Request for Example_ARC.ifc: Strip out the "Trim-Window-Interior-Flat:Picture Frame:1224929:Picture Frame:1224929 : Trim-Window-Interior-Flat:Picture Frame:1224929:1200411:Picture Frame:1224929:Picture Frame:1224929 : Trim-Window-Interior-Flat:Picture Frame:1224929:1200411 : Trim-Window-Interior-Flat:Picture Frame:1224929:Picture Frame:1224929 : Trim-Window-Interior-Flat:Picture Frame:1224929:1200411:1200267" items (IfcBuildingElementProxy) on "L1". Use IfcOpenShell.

First a look at what the model holds.

```python
import ifcopenshell
import ifcopenshell.util.element

model = ifcopenshell.open("Example_ARC.ifc")
print(model.schema)
storey = next(s for s in model.by_type("IfcBuildingStorey") if s.Name == "L1")
proxies = [e for e in ifcopenshell.util.element.get_decomposition(storey) if e.is_a("IfcBuildingElementProxy")]
seen = {}
for e in proxies:
    element_type = ifcopenshell.util.element.get_type(e)
    name = element_type.Name if element_type not in (None, e) else None
    seen[name] = seen.get(name, 0) + 1
for name, count in sorted(seen.items(), key=str):
    print(count, "x", name)
```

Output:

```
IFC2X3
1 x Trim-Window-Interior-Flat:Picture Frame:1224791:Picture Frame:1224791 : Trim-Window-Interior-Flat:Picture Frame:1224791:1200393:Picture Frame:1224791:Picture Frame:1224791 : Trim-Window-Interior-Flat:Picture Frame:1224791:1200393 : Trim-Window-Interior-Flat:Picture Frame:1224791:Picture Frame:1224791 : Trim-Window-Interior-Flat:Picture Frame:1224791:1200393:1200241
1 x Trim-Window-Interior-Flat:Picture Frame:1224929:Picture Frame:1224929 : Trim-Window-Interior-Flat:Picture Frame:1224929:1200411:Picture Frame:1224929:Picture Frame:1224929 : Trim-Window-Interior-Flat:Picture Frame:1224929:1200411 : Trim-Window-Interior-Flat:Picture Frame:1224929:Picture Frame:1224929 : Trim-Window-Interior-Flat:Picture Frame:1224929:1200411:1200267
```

```python
import ifcopenshell
import ifcopenshell.api.root
import ifcopenshell.util.element

model = ifcopenshell.open("Example_ARC.ifc")

storey = next(s for s in model.by_type("IfcBuildingStorey") if s.Name == "L1")
proxies = [e for e in ifcopenshell.util.element.get_decomposition(storey) if e.is_a("IfcBuildingElementProxy")]
targets = [e for e in proxies if (t := ifcopenshell.util.element.get_type(e)) not in (None, e) and t.Name == "Trim-Window-Interior-Flat:Picture Frame:1224929:Picture Frame:1224929 : Trim-Window-Interior-Flat:Picture Frame:1224929:1200411:Picture Frame:1224929:Picture Frame:1224929 : Trim-Window-Interior-Flat:Picture Frame:1224929:1200411 : Trim-Window-Interior-Flat:Picture Frame:1224929:Picture Frame:1224929 : Trim-Window-Interior-Flat:Picture Frame:1224929:1200411:1200267"]

for e in targets:
    ifcopenshell.api.root.remove_product(model, product=e)
print(len(targets), "removed")

model.write("Example_ARC_rev.ifc")
```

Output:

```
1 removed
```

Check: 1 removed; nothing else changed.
